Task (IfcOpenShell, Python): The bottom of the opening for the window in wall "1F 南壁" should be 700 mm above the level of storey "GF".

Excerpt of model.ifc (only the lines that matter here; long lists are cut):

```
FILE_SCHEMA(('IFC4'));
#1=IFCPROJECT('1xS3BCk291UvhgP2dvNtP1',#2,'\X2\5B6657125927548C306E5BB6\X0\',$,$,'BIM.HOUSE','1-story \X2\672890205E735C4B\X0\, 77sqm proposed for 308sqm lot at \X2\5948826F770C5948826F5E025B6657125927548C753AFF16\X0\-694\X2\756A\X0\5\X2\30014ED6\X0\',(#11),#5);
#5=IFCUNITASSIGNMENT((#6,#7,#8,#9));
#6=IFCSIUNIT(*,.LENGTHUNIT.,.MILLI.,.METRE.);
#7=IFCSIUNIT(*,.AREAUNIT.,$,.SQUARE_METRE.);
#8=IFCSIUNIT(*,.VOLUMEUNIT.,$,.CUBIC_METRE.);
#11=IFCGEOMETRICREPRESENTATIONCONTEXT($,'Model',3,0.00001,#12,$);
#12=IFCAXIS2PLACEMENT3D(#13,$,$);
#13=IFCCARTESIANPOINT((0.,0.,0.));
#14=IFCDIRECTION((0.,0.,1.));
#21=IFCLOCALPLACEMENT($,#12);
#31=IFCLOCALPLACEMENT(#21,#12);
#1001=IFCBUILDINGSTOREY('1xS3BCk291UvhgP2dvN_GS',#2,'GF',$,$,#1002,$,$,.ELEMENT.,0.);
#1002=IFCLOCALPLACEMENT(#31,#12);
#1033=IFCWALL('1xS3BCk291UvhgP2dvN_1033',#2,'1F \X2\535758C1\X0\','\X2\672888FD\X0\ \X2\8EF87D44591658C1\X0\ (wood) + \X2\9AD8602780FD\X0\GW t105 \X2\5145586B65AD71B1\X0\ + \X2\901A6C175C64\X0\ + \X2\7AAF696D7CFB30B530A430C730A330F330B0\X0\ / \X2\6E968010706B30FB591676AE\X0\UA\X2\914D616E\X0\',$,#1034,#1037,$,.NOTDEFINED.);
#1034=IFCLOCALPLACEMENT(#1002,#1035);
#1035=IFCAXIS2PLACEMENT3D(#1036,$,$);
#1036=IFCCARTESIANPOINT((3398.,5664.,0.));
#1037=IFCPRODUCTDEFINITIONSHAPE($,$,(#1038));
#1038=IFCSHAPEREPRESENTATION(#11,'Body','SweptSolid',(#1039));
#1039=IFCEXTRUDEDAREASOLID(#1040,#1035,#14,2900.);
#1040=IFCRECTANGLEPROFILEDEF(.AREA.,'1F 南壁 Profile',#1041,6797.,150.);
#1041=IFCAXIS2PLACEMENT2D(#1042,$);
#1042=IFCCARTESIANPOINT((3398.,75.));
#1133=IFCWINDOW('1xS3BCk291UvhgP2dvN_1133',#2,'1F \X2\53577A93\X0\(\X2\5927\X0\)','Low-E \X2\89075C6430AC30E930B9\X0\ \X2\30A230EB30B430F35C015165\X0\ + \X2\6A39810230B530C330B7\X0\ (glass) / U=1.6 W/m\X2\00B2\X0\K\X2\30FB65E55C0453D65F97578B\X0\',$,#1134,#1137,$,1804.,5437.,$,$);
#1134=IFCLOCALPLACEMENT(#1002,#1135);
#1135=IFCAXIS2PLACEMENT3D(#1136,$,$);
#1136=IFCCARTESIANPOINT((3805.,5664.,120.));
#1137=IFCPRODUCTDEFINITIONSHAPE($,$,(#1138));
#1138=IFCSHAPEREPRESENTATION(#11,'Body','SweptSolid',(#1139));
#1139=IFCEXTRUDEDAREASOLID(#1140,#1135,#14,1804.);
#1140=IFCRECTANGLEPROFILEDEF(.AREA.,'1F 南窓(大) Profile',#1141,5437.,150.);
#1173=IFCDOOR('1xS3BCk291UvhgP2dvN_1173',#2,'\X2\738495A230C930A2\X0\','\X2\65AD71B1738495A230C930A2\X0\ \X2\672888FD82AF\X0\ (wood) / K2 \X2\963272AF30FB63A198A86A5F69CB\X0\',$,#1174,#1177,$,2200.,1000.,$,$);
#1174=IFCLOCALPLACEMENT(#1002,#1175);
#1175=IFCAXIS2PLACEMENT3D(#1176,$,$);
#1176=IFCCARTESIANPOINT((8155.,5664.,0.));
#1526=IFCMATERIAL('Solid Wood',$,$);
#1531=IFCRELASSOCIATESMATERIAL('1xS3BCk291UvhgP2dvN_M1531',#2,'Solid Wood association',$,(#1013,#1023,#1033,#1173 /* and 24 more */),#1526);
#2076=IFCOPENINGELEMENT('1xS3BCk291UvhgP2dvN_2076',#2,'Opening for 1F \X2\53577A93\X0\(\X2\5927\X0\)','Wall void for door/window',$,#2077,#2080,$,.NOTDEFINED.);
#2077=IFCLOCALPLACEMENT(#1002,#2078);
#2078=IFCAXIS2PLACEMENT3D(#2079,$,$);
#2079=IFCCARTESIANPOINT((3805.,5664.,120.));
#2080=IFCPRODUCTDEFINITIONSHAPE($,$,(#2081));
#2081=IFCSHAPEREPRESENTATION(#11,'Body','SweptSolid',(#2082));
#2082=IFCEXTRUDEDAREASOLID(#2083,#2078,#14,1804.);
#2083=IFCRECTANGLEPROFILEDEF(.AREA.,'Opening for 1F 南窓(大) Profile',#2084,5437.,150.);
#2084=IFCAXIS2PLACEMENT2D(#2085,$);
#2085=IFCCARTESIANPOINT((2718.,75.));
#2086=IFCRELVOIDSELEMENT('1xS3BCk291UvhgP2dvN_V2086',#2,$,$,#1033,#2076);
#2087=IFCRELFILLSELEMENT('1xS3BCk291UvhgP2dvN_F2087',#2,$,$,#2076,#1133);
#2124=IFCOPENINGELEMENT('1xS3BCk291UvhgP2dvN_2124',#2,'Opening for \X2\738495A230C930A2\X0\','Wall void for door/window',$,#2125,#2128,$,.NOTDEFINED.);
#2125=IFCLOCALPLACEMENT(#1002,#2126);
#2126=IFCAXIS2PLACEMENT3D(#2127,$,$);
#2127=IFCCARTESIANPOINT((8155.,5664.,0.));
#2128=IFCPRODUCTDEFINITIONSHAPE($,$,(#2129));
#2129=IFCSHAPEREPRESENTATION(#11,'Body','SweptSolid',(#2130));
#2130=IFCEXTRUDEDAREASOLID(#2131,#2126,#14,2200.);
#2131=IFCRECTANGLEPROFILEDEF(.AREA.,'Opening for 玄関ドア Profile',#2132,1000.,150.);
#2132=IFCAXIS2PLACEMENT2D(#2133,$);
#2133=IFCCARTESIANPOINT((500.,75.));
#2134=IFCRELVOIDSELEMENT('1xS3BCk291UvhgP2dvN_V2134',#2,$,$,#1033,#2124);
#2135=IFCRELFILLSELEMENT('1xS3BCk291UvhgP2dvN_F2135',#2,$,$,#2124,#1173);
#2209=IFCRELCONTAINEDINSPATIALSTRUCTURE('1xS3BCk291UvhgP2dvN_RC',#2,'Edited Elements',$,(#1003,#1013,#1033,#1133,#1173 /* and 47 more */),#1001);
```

```python
import numpy as np
import ifcopenshell
import ifcopenshell.api.geometry
import ifcopenshell.geom
import ifcopenshell.util.element
import ifcopenshell.util.placement
import ifcopenshell.util.shape
import ifcopenshell.util.unit

model = ifcopenshell.open("model.ifc")
unit_scale = ifcopenshell.util.unit.calculate_unit_scale(model)

window = model.by_id(1133)
opening = window.FillsVoids[0].RelatingOpeningElement
storey = ifcopenshell.util.element.get_container(window, ifc_class="IfcBuildingStorey")
level = ifcopenshell.util.placement.get_local_placement(storey.ObjectPlacement)[2, 3]

# The opening's origin need not be at the sill, so measure its lowest point.
shape = ifcopenshell.geom.create_shape(ifcopenshell.geom.settings(), opening)
bottom = ifcopenshell.util.shape.get_shape_bottom_elevation(shape, shape.geometry) / unit_scale
dz = level + 700.0 - bottom

shift = np.array([0.0, 0.0, dz])
# The window is not placed relative to its opening, so move both.
for product in (opening, window):
    matrix = ifcopenshell.util.placement.get_local_placement(product.ObjectPlacement)
    matrix[:3, 3] += shift
    ifcopenshell.api.geometry.edit_object_placement(model, product=product, matrix=matrix, is_si=False)

print(f"moved by {dz * unit_scale:+.3f} m")

model.write("model_updated.ifc")
```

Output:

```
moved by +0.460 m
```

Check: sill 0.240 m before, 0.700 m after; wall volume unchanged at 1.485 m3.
